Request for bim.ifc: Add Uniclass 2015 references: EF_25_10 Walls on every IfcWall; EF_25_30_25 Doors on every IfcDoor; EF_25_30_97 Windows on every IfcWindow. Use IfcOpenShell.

First a look at what the model holds.

```python
import ifcopenshell

model = ifcopenshell.open("bim.ifc")
print(model.schema)
print("classifications:", [c.Name for c in model.by_type("IfcClassification")])
for ifc_class in ("IfcDoor", "IfcRoof", "IfcStair", "IfcWall", "IfcWindow"):
    print(ifc_class, len(model.by_type(ifc_class)))
```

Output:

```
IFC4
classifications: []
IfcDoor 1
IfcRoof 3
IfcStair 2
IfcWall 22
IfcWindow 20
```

```python
import ifcopenshell
import ifcopenshell.api.classification

model = ifcopenshell.open("bim.ifc")

system = ifcopenshell.api.classification.add_classification(model, classification="Uniclass 2015")

codes = {
    "IfcWall": ("EF_25_10", "Walls"),
    "IfcDoor": ("EF_25_30_25", "Doors"),
    "IfcWindow": ("EF_25_30_97", "Windows"),
}
for ifc_class, (code, name) in codes.items():
    products = model.by_type(ifc_class)
    ifcopenshell.api.classification.add_reference(
        model, products=products, classification=system, identification=code, name=name
    )
    print(code, len(products))

model.write("bim_v2.ifc")
```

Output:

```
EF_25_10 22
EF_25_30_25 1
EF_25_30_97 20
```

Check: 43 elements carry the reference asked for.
